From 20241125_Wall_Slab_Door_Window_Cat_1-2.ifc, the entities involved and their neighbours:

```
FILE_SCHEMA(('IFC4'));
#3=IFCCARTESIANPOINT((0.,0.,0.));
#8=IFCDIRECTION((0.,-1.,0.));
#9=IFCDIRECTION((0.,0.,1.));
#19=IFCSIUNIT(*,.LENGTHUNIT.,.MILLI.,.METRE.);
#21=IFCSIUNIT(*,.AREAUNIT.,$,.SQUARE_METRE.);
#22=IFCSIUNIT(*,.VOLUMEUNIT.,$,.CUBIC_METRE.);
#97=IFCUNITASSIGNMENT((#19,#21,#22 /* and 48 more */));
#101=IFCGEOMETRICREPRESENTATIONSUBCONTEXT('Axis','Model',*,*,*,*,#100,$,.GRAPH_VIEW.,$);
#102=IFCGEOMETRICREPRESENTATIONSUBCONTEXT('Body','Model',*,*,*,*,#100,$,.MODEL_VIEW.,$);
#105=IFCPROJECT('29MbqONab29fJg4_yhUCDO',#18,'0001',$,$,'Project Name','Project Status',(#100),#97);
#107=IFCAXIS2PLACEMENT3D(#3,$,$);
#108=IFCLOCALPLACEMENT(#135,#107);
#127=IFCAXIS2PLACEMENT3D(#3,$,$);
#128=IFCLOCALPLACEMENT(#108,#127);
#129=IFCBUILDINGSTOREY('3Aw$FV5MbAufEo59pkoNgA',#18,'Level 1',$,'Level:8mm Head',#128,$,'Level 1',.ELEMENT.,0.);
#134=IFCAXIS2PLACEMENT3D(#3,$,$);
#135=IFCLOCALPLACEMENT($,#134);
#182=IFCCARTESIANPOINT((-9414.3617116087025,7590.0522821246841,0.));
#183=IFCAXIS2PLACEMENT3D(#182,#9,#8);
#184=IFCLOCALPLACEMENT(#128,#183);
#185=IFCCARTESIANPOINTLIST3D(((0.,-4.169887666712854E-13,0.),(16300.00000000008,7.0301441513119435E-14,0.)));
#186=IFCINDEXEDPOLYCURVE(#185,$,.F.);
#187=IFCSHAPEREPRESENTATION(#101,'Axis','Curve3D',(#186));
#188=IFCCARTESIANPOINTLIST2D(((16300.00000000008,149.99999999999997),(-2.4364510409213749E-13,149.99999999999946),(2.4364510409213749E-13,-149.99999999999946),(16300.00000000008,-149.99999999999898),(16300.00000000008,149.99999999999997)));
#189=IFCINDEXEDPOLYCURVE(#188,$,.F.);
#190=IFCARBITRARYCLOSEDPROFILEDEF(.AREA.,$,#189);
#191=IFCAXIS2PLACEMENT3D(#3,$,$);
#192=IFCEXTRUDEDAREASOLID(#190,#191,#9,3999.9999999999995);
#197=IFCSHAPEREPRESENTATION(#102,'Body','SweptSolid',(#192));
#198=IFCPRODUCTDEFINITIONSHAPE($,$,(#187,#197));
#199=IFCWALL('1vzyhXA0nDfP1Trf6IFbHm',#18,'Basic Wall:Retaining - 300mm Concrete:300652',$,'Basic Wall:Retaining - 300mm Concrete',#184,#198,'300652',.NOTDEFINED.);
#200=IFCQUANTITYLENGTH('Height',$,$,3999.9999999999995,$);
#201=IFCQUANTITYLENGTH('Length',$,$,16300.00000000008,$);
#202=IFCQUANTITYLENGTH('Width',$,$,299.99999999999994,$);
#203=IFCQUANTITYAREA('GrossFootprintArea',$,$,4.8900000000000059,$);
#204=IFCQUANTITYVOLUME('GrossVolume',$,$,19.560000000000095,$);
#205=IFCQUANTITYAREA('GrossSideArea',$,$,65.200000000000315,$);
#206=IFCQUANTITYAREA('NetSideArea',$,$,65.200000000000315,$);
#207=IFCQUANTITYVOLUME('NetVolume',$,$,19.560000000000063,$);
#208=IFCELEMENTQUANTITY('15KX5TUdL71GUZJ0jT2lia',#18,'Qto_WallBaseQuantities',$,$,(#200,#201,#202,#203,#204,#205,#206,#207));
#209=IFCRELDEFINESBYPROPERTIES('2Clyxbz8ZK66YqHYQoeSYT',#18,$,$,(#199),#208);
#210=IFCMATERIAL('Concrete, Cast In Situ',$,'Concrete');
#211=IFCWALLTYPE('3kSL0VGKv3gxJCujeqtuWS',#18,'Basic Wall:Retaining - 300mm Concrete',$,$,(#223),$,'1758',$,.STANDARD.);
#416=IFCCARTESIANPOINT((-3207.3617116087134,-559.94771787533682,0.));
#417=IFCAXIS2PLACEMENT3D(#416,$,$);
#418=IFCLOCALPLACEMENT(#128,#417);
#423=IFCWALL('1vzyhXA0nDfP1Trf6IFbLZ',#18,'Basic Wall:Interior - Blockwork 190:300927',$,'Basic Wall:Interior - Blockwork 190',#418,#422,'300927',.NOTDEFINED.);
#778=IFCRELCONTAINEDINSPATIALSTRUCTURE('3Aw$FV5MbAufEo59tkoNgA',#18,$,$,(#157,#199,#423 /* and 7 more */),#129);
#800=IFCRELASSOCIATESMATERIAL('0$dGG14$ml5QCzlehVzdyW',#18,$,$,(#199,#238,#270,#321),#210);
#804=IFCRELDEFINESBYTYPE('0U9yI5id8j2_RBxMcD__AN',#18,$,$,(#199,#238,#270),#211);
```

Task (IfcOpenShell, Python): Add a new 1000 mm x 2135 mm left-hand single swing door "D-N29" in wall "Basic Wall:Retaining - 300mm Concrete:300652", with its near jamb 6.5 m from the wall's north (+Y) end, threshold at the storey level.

```python
import numpy as np
import ifcopenshell
import ifcopenshell.api.feature
import ifcopenshell.api.geometry
import ifcopenshell.api.pset
import ifcopenshell.api.root
import ifcopenshell.api.spatial
import ifcopenshell.geom
import ifcopenshell.util.element
import ifcopenshell.util.placement
import ifcopenshell.util.representation
import ifcopenshell.util.shape
import ifcopenshell.util.unit

model = ifcopenshell.open("20241125_Wall_Slab_Door_Window_Cat_1-2.ifc")
unit_scale = ifcopenshell.util.unit.calculate_unit_scale(model)
area_scale = ifcopenshell.util.unit.calculate_unit_scale(model, "AREAUNIT")
volume_scale = ifcopenshell.util.unit.calculate_unit_scale(model, "VOLUMEUNIT")
settings = ifcopenshell.geom.settings()


def volume(element):
    """Net volume in cubic metres, openings subtracted."""
    shape = ifcopenshell.geom.create_shape(settings, element)
    return ifcopenshell.util.shape.get_volume(shape.geometry)


wall = model.by_guid("1vzyhXA0nDfP1Trf6IFbHm")
storey = ifcopenshell.util.element.get_container(wall, ifc_class="IfcBuildingStorey")
context = ifcopenshell.util.representation.get_context(model, "Model", "Body", "MODEL_VIEW")
before = volume(wall)

width, height, from_end, sill = 1, 2.135, 6.5, 0.0  # metres

# The wall runs along its own X axis, and the end named is its -X end.
wall_shape = ifcopenshell.geom.create_shape(settings, wall)
x, y, z = ifcopenshell.util.shape.get_vertices(wall_shape.geometry).T
start = x.min() + from_end
face, thickness = float(y.min()), float(y.max() - y.min())
wall_matrix = ifcopenshell.util.placement.get_local_placement(wall.ObjectPlacement)
level = ifcopenshell.util.placement.get_local_placement(storey.ObjectPlacement)[2, 3]


def in_wall(x, y):
    """Placement at x, y metres in the wall's axes, at sill height."""
    matrix = wall_matrix.copy()
    matrix[:, 3] = wall_matrix @ np.array([x / unit_scale, y / unit_scale, 0.0, 1.0])
    matrix[2, 3] = level + sill / unit_scale
    return matrix


# Opening: a box that overshoots both wall faces by 50 mm.
opening = ifcopenshell.api.root.create_entity(model, ifc_class="IfcOpeningElement", predefined_type="OPENING")
box = ifcopenshell.api.geometry.add_wall_representation(
    model, context=context, length=width, height=height, thickness=thickness + 0.1
)
ifcopenshell.api.geometry.assign_representation(model, product=opening, representation=box)
ifcopenshell.api.geometry.edit_object_placement(model, product=opening, matrix=in_wall(start, face - 0.05), is_si=False)
ifcopenshell.api.feature.add_feature(model, feature=opening, element=wall)

door = ifcopenshell.api.root.create_entity(model, ifc_class="IfcDoor", name="D-N29", predefined_type="DOOR")
door.OverallWidth, door.OverallHeight = width / unit_scale, height / unit_scale
door.OperationType = "SINGLE_SWING_LEFT"
body = ifcopenshell.api.geometry.add_door_representation(
    model,
    context=context,
    overall_width=door.OverallWidth,
    overall_height=door.OverallHeight,
    operation_type="SINGLE_SWING_LEFT",
    lining_properties={"LiningDepth": thickness / unit_scale, "ThresholdDepth": thickness / unit_scale},
)
ifcopenshell.api.geometry.assign_representation(model, product=door, representation=body)
ifcopenshell.api.spatial.assign_container(model, products=[door], relating_structure=storey)
ifcopenshell.api.feature.add_filling(model, opening=opening, element=door)

# The lining spans the wall, so the door starts at the wall face.
ifcopenshell.api.geometry.edit_object_placement(model, product=door, matrix=in_wall(start, face), is_si=False)

after = volume(wall)

# Update the wall's stored quantities.
qto = model.by_id(ifcopenshell.util.element.get_pset(wall, "Qto_WallBaseQuantities", should_inherit=False)["id"])
ifcopenshell.api.pset.edit_qto(model, qto=qto, properties={
    "NetSideArea": after / thickness / area_scale,
    "NetVolume": after / volume_scale,
})

print(f"wall volume {before:.3f} -> {after:.3f} m3")

model.write("20241125_Wall_Slab_Door_Window_Cat_1-2-out.ifc")
```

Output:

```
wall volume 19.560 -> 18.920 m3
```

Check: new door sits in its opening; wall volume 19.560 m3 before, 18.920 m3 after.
